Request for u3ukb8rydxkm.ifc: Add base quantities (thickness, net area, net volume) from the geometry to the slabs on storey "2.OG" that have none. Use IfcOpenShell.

First a look at what the model holds.

```python
import ifcopenshell
import ifcopenshell.util.element
import ifcopenshell.util.unit

model = ifcopenshell.open("u3ukb8rydxkm.ifc")
print(model.schema)
for unit_type in ("LENGTHUNIT", "AREAUNIT", "VOLUMEUNIT"):
    print(unit_type, ifcopenshell.util.unit.calculate_unit_scale(model, unit_type))
storey = next(s for s in model.by_type("IfcBuildingStorey") if s.Name == "2.OG")
slabs = [e for e in ifcopenshell.util.element.get_decomposition(storey) if e.is_a("IfcSlab")]
for e in sorted(slabs, key=lambda e: e.id()):
    print(e.id(), e.is_a(), e.Name, list(ifcopenshell.util.element.get_psets(e, qtos_only=True)), sep=" | ")
```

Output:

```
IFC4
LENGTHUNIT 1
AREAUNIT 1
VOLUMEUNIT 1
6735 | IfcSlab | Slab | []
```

```python
import ifcopenshell
import ifcopenshell.api.pset
import ifcopenshell.geom
import ifcopenshell.util.element
import ifcopenshell.util.shape
import ifcopenshell.util.unit

model = ifcopenshell.open("u3ukb8rydxkm.ifc")
unit_scale = ifcopenshell.util.unit.calculate_unit_scale(model)
area_scale = ifcopenshell.util.unit.calculate_unit_scale(model, "AREAUNIT")
volume_scale = ifcopenshell.util.unit.calculate_unit_scale(model, "VOLUMEUNIT")
settings = ifcopenshell.geom.settings()

storey = next(s for s in model.by_type("IfcBuildingStorey") if s.Name == "2.OG")
slabs = [e for e in ifcopenshell.util.element.get_decomposition(storey) if e.is_a("IfcSlab")]

for e in sorted(slabs, key=lambda e: e.id()):
    if ifcopenshell.util.element.get_psets(e, qtos_only=True, should_inherit=False):
        continue
    # Geometry comes back in metres, in the element's own axes.
    shape = ifcopenshell.geom.create_shape(settings, e)
    values = {
        "Width": ifcopenshell.util.shape.get_z(shape.geometry) / unit_scale,
        "NetArea": ifcopenshell.util.shape.get_footprint_area(shape.geometry) / area_scale,
        "NetVolume": ifcopenshell.util.shape.get_volume(shape.geometry) / volume_scale,
    }
    qto = ifcopenshell.api.pset.add_qto(model, product=e, name="Qto_SlabBaseQuantities")
    ifcopenshell.api.pset.edit_qto(model, qto=qto, properties=values)
    print(e.id(), {k: round(v, 3) for k, v in values.items()})

model.write("u3ukb8rydxkm_v2.ifc")
```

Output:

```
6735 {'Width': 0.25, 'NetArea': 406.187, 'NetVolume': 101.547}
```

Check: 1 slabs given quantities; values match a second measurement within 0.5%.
